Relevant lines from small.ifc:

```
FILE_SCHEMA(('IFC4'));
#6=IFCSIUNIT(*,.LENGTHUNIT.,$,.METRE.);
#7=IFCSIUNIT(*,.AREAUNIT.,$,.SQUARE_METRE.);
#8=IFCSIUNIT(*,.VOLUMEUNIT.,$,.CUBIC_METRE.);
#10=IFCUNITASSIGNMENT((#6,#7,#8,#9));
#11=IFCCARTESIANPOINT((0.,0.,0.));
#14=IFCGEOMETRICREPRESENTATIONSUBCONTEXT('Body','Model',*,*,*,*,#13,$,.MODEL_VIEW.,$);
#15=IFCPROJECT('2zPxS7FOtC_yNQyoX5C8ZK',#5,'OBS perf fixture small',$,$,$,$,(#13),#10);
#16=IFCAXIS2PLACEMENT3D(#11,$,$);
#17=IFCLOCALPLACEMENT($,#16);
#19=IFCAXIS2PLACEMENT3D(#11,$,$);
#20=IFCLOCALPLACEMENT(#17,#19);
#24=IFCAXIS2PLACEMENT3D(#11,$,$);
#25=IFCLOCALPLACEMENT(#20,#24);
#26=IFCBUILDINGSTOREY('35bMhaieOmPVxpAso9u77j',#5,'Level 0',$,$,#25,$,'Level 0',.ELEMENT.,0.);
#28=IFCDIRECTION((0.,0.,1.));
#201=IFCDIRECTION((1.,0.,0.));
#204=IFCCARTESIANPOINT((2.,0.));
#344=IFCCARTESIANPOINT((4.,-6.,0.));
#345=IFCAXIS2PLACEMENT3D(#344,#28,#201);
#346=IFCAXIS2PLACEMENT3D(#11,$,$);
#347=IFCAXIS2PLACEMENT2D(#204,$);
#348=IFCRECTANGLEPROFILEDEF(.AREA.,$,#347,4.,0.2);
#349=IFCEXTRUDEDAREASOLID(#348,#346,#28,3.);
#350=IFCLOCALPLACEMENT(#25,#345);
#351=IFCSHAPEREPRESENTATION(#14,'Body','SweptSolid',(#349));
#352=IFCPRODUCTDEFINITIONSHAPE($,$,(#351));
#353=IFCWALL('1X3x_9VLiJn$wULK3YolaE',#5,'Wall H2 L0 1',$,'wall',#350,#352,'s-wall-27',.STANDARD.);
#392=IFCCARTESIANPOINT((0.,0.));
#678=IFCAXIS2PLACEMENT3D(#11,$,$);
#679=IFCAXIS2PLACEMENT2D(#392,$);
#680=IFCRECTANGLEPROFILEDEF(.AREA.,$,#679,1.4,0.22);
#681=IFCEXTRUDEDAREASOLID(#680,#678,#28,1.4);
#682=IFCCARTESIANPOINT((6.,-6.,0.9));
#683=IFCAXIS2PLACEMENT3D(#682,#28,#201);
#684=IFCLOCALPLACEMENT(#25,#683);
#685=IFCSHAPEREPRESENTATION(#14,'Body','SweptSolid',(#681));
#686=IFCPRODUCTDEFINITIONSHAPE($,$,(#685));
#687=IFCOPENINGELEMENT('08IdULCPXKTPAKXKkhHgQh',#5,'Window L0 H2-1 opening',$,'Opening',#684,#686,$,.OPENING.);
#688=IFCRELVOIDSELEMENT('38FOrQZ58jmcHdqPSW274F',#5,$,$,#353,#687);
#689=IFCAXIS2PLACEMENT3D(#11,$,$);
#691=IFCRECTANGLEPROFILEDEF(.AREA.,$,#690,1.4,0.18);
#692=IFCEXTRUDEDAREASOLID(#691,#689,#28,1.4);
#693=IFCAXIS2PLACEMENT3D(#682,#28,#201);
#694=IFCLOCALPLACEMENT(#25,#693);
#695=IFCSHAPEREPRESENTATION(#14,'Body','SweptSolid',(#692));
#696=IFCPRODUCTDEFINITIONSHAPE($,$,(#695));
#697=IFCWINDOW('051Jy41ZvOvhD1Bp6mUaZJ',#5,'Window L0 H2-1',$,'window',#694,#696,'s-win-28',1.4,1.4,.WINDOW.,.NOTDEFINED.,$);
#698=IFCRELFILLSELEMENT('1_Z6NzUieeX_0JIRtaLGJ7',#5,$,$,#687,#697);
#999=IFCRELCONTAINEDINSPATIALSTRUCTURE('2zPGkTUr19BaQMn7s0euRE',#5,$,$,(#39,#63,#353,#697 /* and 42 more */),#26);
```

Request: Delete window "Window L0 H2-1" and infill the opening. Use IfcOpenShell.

```python
import ifcopenshell
import ifcopenshell.api.feature
import ifcopenshell.api.root
import ifcopenshell.geom
import ifcopenshell.util.shape

model = ifcopenshell.open("small.ifc")
settings = ifcopenshell.geom.settings()


def volume(element):
    """Net volume in cubic metres, openings subtracted."""
    shape = ifcopenshell.geom.create_shape(settings, element)
    return ifcopenshell.util.shape.get_volume(shape.geometry)


window = model.by_id(697)
opening = window.FillsVoids[0].RelatingOpeningElement
wall = opening.VoidsElements[0].RelatingBuildingElement
before = volume(wall)

ifcopenshell.api.root.remove_product(model, product=window)
ifcopenshell.api.feature.remove_feature(model, feature=opening)

after = volume(wall)

print(f"wall volume {before:.3f} -> {after:.3f} m3")

model.write("small_edited.ifc")
```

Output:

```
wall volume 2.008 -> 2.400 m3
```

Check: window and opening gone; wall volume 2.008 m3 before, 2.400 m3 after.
